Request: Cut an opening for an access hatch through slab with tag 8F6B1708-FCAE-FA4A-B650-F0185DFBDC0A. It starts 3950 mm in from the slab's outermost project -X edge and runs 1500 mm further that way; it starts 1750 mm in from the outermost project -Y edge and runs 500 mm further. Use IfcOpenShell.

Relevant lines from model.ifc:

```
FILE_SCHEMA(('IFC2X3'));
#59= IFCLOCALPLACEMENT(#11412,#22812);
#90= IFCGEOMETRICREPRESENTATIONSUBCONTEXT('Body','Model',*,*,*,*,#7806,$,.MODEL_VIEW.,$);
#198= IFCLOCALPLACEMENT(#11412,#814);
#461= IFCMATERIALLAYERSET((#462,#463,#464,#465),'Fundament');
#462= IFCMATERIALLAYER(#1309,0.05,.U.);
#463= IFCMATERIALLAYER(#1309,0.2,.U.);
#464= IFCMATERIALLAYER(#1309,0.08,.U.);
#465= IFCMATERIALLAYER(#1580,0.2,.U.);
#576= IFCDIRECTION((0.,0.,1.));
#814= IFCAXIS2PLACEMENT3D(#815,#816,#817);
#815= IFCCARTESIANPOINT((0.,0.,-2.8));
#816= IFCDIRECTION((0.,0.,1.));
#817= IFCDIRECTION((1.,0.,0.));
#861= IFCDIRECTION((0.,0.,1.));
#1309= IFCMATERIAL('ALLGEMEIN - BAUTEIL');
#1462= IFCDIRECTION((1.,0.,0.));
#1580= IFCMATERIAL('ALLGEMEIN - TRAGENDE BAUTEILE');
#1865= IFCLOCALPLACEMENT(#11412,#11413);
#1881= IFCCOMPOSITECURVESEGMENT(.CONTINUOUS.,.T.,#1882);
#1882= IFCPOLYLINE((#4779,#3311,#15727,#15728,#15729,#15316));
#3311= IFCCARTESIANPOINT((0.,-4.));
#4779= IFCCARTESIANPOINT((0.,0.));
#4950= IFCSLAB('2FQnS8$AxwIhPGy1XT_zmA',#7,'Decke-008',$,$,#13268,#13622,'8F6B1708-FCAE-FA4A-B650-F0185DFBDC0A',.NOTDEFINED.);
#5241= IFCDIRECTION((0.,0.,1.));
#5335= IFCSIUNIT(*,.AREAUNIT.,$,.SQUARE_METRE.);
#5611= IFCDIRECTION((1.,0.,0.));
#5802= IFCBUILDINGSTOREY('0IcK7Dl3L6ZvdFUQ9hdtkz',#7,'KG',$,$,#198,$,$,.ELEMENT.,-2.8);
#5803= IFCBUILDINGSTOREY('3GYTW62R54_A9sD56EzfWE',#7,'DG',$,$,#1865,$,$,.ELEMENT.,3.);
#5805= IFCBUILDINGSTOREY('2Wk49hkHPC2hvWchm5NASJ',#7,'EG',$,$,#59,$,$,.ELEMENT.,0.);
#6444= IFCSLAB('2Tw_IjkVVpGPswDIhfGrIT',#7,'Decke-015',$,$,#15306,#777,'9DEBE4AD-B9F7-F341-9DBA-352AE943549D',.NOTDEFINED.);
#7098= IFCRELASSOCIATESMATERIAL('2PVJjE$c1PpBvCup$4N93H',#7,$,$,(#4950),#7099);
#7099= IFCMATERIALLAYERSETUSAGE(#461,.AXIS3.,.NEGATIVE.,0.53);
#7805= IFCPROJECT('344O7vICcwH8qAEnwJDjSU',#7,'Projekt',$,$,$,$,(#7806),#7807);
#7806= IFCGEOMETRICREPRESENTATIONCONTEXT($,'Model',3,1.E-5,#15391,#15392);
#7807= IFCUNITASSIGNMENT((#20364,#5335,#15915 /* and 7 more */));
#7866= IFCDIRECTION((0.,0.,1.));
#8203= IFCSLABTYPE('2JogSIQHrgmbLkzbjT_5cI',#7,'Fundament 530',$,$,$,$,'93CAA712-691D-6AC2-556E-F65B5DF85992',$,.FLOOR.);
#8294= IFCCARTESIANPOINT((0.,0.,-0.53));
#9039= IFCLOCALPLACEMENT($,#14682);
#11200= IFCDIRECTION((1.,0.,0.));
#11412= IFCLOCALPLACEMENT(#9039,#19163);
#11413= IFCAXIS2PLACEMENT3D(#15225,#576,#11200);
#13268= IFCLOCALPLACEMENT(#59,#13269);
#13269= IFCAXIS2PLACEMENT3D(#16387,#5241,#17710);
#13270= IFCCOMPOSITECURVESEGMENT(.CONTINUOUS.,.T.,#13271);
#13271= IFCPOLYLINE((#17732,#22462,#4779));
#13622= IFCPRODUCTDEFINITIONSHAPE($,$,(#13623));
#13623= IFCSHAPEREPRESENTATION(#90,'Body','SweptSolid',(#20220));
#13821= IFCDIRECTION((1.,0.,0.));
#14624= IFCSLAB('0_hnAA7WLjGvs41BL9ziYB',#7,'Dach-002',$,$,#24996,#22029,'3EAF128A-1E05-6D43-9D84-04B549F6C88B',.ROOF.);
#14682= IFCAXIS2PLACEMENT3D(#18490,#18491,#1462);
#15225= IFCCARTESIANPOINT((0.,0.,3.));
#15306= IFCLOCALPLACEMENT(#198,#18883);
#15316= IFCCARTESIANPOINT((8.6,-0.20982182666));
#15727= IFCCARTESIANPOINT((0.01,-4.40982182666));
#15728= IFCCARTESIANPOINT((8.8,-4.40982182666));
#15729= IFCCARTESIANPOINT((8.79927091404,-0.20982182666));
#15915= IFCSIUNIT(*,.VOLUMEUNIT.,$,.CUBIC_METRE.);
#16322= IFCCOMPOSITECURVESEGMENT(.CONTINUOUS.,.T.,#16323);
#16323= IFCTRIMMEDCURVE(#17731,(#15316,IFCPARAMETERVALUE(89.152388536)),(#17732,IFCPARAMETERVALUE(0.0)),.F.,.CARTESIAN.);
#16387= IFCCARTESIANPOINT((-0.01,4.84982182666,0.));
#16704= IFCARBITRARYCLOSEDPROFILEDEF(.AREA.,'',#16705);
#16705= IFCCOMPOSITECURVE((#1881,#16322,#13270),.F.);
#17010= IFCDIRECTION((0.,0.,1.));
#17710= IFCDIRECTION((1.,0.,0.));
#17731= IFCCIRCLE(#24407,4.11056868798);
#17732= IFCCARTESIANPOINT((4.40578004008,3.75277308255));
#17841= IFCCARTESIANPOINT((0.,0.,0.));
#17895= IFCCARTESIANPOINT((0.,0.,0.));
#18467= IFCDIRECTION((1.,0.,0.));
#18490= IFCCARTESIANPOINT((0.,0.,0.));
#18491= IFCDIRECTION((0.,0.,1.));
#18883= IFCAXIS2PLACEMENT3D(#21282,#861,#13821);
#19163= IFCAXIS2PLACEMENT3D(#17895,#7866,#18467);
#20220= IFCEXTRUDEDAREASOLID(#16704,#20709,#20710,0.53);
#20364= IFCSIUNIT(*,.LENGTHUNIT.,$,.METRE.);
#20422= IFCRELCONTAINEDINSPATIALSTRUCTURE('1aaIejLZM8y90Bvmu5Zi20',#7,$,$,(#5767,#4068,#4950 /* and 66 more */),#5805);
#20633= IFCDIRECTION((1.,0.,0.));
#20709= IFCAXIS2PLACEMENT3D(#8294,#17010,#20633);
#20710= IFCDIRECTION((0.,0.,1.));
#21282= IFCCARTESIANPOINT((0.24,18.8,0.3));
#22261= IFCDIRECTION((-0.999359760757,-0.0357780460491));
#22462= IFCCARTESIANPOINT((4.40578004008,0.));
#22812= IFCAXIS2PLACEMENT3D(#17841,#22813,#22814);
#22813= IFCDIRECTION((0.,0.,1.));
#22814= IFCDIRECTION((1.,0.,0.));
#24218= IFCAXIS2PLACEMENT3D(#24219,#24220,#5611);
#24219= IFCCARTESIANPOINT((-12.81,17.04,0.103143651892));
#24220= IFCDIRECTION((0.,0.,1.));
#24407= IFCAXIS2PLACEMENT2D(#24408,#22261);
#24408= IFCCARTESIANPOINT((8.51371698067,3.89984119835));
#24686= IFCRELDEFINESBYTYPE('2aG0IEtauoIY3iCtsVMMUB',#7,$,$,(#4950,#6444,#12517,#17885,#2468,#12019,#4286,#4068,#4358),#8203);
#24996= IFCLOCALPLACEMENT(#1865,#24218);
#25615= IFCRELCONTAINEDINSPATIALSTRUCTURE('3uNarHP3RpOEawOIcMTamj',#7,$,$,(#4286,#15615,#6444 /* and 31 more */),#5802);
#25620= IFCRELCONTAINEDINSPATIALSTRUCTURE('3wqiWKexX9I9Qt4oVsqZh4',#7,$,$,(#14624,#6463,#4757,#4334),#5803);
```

```python
import numpy as np
import ifcopenshell
import ifcopenshell.api.feature
import ifcopenshell.api.geometry
import ifcopenshell.api.root
import ifcopenshell.geom
import ifcopenshell.util.placement
import ifcopenshell.util.representation
import ifcopenshell.util.shape
import ifcopenshell.util.unit

model = ifcopenshell.open("model.ifc")
unit_scale = ifcopenshell.util.unit.calculate_unit_scale(model)
settings = ifcopenshell.geom.settings()


def volume(element):
    """Net volume in cubic metres, openings subtracted."""
    shape = ifcopenshell.geom.create_shape(settings, element)
    return ifcopenshell.util.shape.get_volume(shape.geometry)


slab = model.by_id(4950)
before = volume(slab)

# Extent in the slab's own axes, in metres. The edges named are its -X and -Y sides.
slab_shape = ifcopenshell.geom.create_shape(settings, slab)
vertices = ifcopenshell.util.shape.get_vertices(slab_shape.geometry)
x_min, y_min, bottom = vertices.min(axis=0)
top = vertices[:, 2].max()

opening = ifcopenshell.api.root.create_entity(model, ifc_class="IfcOpeningElement", name="Access hatch opening")
context = ifcopenshell.util.representation.get_context(model, "Model", "Body", "MODEL_VIEW")
width, depth = 1.5, 0.5
outline = [(0.0, 0.0), (width, 0.0), (width, depth), (0.0, depth), (0.0, 0.0)]
# Overshoot both faces by 50 mm so the cut is clean.
shape = ifcopenshell.api.geometry.add_slab_representation(
    model, context=context, depth=top - bottom + 0.1, polyline=outline
)
ifcopenshell.api.geometry.assign_representation(model, product=opening, representation=shape)

matrix = ifcopenshell.util.placement.get_local_placement(slab.ObjectPlacement)
matrix[:, 3] = matrix @ np.append(np.array([x_min + 3.95, y_min + 1.75, bottom - 0.05]) / unit_scale, 1.0)
ifcopenshell.api.geometry.edit_object_placement(model, product=opening, matrix=matrix, is_si=False)
ifcopenshell.api.feature.add_feature(model, feature=opening, element=slab)

after = volume(slab)

print(f"slab volume {before:.3f} -> {after:.3f} m3")

model.write("model_edited.ifc")
```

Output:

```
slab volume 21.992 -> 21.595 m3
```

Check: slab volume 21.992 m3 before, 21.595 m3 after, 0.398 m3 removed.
